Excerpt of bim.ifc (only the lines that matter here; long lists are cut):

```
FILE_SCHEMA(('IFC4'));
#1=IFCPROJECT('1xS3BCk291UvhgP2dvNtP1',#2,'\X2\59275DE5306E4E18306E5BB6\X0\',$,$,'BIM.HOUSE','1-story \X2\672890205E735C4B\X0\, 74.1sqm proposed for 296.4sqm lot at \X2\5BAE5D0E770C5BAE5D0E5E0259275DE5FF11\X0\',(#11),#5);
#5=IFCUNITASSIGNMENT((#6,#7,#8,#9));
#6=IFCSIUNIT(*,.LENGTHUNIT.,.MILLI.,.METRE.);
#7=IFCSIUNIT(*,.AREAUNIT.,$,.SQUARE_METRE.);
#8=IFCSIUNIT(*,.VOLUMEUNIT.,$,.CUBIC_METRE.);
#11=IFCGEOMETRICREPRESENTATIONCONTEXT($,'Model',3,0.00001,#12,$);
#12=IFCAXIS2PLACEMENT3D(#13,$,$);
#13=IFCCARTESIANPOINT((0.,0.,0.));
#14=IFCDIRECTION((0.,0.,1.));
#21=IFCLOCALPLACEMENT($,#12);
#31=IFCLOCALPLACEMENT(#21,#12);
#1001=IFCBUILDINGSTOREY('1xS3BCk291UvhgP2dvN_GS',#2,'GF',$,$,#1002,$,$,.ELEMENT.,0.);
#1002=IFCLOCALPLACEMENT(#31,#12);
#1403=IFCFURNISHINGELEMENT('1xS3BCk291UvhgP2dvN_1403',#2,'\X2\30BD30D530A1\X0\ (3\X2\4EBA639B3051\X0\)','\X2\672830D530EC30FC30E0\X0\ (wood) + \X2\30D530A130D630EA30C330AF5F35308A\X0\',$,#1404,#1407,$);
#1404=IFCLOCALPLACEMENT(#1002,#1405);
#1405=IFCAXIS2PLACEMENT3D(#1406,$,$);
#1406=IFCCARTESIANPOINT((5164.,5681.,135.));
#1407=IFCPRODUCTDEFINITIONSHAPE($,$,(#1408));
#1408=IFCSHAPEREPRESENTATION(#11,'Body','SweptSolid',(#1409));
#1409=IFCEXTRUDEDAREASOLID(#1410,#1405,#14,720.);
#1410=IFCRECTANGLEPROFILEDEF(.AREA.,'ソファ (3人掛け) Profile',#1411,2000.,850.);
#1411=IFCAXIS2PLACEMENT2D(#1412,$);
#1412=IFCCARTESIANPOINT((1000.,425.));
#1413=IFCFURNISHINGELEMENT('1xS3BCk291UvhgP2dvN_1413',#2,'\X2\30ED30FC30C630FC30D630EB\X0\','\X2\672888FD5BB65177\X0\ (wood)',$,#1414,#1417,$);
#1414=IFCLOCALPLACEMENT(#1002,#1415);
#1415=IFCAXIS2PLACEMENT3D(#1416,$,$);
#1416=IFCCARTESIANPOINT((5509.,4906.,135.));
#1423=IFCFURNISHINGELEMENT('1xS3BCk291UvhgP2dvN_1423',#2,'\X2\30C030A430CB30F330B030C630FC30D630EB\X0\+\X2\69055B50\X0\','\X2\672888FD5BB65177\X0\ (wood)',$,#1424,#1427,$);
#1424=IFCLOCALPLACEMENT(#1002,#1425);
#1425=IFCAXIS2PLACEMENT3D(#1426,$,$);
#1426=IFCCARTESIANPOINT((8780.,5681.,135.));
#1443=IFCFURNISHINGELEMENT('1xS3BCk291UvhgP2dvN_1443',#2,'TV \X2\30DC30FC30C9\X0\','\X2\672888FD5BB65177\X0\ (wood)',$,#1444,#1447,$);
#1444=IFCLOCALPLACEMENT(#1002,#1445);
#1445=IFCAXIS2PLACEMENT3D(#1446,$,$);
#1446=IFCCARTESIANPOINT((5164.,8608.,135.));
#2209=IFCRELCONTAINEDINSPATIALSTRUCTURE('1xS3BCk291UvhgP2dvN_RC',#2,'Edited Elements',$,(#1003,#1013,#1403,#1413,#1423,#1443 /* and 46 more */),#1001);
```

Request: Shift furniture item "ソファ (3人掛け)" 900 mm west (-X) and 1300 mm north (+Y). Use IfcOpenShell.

```python
import ifcopenshell
import ifcopenshell.api.geometry
import ifcopenshell.util.placement
import ifcopenshell.util.unit

model = ifcopenshell.open("bim.ifc")
unit_scale = ifcopenshell.util.unit.calculate_unit_scale(model)

item = model.by_id(1403)
matrix = ifcopenshell.util.placement.get_local_placement(item.ObjectPlacement)
matrix[0, 3] -= 0.9 / unit_scale
matrix[1, 3] += 1.3 / unit_scale
ifcopenshell.api.geometry.edit_object_placement(model, product=item, matrix=matrix, is_si=False)

print(ifcopenshell.util.placement.get_local_placement(item.ObjectPlacement).round(3) + 0.0)

model.write("bim_rev.ifc")
```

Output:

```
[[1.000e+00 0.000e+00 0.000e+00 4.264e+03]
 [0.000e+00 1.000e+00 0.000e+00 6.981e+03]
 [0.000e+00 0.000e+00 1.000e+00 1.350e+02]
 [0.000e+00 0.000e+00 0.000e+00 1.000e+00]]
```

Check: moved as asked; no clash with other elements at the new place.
